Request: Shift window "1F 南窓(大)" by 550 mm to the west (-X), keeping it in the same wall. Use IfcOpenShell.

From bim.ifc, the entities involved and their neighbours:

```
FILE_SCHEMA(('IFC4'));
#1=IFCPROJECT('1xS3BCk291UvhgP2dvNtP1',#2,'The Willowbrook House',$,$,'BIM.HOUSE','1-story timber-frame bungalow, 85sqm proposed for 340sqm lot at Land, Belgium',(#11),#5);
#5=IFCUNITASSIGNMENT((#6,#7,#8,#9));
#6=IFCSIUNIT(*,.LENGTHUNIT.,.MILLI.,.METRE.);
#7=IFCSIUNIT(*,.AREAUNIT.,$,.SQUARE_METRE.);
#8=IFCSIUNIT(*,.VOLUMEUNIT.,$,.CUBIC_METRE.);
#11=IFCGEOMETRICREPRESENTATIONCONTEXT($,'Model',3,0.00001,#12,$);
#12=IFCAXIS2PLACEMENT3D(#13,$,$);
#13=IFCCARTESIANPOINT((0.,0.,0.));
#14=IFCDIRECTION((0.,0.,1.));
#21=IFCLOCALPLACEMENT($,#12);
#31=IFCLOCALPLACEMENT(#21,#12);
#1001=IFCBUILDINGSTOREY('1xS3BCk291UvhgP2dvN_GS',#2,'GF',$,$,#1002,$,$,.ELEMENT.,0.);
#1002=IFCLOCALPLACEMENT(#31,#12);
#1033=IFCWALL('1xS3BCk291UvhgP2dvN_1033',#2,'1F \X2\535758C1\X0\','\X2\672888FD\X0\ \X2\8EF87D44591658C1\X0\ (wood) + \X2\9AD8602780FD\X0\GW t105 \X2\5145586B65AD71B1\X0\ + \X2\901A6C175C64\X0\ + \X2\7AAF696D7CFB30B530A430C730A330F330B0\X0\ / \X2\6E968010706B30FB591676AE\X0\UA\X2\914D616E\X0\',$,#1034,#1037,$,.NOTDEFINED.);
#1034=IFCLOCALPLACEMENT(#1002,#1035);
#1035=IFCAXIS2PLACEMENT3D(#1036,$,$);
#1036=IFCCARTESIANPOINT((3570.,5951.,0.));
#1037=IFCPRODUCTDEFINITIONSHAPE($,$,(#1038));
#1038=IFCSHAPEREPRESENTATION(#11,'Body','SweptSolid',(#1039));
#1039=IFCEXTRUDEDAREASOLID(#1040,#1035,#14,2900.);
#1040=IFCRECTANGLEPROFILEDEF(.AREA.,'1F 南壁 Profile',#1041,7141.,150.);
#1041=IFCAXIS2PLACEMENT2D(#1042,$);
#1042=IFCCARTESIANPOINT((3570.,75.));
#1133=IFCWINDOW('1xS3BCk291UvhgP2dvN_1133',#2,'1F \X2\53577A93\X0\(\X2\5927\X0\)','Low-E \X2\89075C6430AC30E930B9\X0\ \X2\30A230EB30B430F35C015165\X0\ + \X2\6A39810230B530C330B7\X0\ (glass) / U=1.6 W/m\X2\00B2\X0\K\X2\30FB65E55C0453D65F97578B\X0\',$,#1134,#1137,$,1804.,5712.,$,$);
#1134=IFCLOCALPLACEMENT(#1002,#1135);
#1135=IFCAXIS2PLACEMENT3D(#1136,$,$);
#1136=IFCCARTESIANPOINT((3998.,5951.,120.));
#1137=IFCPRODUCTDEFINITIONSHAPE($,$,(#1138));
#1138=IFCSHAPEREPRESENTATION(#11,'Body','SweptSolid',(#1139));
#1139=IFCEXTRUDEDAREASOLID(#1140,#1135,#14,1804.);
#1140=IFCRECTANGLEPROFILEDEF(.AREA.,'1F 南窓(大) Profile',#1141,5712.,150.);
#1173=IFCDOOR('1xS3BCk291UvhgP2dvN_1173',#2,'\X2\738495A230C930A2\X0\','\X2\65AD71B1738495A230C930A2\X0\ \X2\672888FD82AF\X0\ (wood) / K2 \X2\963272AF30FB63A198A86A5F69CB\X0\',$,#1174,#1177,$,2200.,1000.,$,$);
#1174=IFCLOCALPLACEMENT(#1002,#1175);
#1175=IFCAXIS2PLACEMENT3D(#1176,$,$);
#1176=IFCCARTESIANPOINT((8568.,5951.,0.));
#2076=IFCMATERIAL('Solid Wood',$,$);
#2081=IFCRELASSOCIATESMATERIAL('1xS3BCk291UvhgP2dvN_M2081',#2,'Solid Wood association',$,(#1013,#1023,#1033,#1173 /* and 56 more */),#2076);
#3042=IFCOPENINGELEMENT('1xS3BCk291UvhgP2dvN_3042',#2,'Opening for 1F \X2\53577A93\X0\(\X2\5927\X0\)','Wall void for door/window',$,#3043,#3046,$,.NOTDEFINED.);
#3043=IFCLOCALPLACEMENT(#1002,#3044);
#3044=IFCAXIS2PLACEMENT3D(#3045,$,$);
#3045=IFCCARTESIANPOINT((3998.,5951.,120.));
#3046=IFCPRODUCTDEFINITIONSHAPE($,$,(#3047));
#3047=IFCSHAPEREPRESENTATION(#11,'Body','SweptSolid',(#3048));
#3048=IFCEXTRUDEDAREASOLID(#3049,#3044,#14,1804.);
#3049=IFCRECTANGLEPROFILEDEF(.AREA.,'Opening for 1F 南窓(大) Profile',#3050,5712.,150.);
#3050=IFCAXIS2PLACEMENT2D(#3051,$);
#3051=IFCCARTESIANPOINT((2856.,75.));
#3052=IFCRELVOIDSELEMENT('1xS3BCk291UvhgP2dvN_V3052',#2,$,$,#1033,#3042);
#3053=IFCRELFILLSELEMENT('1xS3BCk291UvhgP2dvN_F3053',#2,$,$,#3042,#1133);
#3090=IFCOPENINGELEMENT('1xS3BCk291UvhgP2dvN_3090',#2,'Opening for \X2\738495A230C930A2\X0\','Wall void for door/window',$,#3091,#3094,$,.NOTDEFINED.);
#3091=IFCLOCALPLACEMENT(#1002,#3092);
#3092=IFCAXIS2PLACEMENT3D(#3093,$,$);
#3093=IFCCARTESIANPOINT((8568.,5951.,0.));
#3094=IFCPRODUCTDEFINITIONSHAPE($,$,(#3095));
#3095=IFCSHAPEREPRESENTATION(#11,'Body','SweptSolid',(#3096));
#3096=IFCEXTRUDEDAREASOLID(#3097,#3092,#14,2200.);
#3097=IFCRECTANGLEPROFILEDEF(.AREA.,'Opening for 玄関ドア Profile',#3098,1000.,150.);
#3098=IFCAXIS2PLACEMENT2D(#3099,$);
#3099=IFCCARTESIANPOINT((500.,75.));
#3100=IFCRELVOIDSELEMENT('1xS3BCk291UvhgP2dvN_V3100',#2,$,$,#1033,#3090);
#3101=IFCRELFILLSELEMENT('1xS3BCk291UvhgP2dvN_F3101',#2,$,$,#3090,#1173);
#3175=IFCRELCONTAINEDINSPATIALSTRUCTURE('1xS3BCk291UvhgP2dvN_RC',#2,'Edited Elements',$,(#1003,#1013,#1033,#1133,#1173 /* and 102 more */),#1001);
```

```python
import ifcopenshell
import ifcopenshell.api.geometry
import ifcopenshell.util.placement
import ifcopenshell.util.unit

model = ifcopenshell.open("bim.ifc")
unit_scale = ifcopenshell.util.unit.calculate_unit_scale(model)

window = model.by_guid("1xS3BCk291UvhgP2dvN_1133")
opening = window.FillsVoids[0].RelatingOpeningElement
wall = opening.VoidsElements[0].RelatingBuildingElement

wall_matrix = ifcopenshell.util.placement.get_local_placement(wall.ObjectPlacement)
shift = wall_matrix[:3, 0] * -0.55 / unit_scale
before = ifcopenshell.util.placement.get_local_placement(window.ObjectPlacement)[:3, 3].copy()

# The window is not placed relative to its opening, so move both.
for product in (opening, window):
    matrix = ifcopenshell.util.placement.get_local_placement(product.ObjectPlacement)
    matrix[:3, 3] += shift
    ifcopenshell.api.geometry.edit_object_placement(model, product=product, matrix=matrix, is_si=False)

after = ifcopenshell.util.placement.get_local_placement(window.ObjectPlacement)[:3, 3]
print("window moved by", (after - before).round(3) + 0.0)

model.write("bim-out.ifc")
```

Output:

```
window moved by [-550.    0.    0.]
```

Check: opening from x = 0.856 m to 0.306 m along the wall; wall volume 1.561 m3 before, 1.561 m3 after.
